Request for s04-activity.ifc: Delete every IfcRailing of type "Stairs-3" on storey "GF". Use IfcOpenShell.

First a look at what the model holds.

```python
import ifcopenshell
import ifcopenshell.util.element

model = ifcopenshell.open("s04-activity.ifc")
print(model.schema)
storey = next(s for s in model.by_type("IfcBuildingStorey") if s.Name == "GF")
railings = [e for e in ifcopenshell.util.element.get_decomposition(storey) if e.is_a("IfcRailing")]
seen = {}
for e in railings:
    element_type = ifcopenshell.util.element.get_type(e)
    name = element_type.Name if element_type not in (None, e) else None
    seen[name] = seen.get(name, 0) + 1
for name, count in sorted(seen.items(), key=str):
    print(count, "x", name)
```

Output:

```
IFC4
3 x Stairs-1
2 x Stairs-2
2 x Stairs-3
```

```python
import ifcopenshell
import ifcopenshell.api.root
import ifcopenshell.util.element

model = ifcopenshell.open("s04-activity.ifc")

storey = next(s for s in model.by_type("IfcBuildingStorey") if s.Name == "GF")
railings = [e for e in ifcopenshell.util.element.get_decomposition(storey) if e.is_a("IfcRailing")]
targets = [e for e in railings if (t := ifcopenshell.util.element.get_type(e)) not in (None, e) and t.Name == "Stairs-3"]

for e in targets:
    ifcopenshell.api.root.remove_product(model, product=e)
print(len(targets), "removed")

model.write("s04-activity_rev.ifc")
```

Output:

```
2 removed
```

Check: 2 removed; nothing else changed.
